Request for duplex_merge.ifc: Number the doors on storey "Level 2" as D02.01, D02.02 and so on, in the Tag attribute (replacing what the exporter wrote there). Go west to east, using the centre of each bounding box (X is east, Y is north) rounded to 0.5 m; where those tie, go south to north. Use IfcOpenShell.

First a look at what the model holds.

```python
import ifcopenshell
import ifcopenshell.util.element
import ifcopenshell.util.placement

model = ifcopenshell.open("duplex_merge.ifc")
print(model.schema)
storey = next(s for s in model.by_type("IfcBuildingStorey") if s.Name == "Level 2")
doors = [e for e in ifcopenshell.util.element.get_decomposition(storey) if e.is_a("IfcDoor")]
for e in sorted(doors, key=lambda e: e.id()):
    origin = ifcopenshell.util.placement.get_local_placement(e.ObjectPlacement)[:3, 3]
    print(e.id(), e.Tag, e.Name, origin.round(2) + 0.0, sep=" | ")
```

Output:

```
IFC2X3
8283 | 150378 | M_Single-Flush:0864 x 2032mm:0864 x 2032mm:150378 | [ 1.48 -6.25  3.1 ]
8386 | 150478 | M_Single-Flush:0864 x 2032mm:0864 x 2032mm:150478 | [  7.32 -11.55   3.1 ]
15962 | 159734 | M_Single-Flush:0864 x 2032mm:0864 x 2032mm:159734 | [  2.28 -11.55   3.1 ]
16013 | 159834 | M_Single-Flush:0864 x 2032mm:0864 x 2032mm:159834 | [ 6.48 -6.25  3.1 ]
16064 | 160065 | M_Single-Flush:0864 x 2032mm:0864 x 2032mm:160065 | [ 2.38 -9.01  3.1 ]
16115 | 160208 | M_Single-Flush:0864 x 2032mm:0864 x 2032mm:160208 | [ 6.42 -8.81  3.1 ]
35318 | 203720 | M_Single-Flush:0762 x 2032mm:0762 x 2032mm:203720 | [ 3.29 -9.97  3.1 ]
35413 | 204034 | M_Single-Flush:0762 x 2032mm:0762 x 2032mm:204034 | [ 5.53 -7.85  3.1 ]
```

```python
import ifcopenshell
import ifcopenshell.geom
import ifcopenshell.util.element
import ifcopenshell.util.shape

model = ifcopenshell.open("duplex_merge.ifc")
settings = ifcopenshell.geom.settings()
settings.set("use-world-coords", True)


def centre(element):
    shape = ifcopenshell.geom.create_shape(settings, element)
    return ifcopenshell.util.shape.get_bbox_centroid(shape.geometry)


storey = next(s for s in model.by_type("IfcBuildingStorey") if s.Name == "Level 2")
doors = [e for e in ifcopenshell.util.element.get_decomposition(storey) if e.is_a("IfcDoor")]

# Insertion points can sit at a corner or the storey origin, so sort by the geometry (in metres).
centres = {e: centre(e) for e in doors}
doors.sort(key=lambda e: (round(centres[e][0] / 0.5), centres[e][1]))

for i, e in enumerate(doors, start=1):
    number = f"D02.{i:02d}"
    e.Tag = number
    print(e.id(), number)

model.write("duplex_merge-out.ifc")
```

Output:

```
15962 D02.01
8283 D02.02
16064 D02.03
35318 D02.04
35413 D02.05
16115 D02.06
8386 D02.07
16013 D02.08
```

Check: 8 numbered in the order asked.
